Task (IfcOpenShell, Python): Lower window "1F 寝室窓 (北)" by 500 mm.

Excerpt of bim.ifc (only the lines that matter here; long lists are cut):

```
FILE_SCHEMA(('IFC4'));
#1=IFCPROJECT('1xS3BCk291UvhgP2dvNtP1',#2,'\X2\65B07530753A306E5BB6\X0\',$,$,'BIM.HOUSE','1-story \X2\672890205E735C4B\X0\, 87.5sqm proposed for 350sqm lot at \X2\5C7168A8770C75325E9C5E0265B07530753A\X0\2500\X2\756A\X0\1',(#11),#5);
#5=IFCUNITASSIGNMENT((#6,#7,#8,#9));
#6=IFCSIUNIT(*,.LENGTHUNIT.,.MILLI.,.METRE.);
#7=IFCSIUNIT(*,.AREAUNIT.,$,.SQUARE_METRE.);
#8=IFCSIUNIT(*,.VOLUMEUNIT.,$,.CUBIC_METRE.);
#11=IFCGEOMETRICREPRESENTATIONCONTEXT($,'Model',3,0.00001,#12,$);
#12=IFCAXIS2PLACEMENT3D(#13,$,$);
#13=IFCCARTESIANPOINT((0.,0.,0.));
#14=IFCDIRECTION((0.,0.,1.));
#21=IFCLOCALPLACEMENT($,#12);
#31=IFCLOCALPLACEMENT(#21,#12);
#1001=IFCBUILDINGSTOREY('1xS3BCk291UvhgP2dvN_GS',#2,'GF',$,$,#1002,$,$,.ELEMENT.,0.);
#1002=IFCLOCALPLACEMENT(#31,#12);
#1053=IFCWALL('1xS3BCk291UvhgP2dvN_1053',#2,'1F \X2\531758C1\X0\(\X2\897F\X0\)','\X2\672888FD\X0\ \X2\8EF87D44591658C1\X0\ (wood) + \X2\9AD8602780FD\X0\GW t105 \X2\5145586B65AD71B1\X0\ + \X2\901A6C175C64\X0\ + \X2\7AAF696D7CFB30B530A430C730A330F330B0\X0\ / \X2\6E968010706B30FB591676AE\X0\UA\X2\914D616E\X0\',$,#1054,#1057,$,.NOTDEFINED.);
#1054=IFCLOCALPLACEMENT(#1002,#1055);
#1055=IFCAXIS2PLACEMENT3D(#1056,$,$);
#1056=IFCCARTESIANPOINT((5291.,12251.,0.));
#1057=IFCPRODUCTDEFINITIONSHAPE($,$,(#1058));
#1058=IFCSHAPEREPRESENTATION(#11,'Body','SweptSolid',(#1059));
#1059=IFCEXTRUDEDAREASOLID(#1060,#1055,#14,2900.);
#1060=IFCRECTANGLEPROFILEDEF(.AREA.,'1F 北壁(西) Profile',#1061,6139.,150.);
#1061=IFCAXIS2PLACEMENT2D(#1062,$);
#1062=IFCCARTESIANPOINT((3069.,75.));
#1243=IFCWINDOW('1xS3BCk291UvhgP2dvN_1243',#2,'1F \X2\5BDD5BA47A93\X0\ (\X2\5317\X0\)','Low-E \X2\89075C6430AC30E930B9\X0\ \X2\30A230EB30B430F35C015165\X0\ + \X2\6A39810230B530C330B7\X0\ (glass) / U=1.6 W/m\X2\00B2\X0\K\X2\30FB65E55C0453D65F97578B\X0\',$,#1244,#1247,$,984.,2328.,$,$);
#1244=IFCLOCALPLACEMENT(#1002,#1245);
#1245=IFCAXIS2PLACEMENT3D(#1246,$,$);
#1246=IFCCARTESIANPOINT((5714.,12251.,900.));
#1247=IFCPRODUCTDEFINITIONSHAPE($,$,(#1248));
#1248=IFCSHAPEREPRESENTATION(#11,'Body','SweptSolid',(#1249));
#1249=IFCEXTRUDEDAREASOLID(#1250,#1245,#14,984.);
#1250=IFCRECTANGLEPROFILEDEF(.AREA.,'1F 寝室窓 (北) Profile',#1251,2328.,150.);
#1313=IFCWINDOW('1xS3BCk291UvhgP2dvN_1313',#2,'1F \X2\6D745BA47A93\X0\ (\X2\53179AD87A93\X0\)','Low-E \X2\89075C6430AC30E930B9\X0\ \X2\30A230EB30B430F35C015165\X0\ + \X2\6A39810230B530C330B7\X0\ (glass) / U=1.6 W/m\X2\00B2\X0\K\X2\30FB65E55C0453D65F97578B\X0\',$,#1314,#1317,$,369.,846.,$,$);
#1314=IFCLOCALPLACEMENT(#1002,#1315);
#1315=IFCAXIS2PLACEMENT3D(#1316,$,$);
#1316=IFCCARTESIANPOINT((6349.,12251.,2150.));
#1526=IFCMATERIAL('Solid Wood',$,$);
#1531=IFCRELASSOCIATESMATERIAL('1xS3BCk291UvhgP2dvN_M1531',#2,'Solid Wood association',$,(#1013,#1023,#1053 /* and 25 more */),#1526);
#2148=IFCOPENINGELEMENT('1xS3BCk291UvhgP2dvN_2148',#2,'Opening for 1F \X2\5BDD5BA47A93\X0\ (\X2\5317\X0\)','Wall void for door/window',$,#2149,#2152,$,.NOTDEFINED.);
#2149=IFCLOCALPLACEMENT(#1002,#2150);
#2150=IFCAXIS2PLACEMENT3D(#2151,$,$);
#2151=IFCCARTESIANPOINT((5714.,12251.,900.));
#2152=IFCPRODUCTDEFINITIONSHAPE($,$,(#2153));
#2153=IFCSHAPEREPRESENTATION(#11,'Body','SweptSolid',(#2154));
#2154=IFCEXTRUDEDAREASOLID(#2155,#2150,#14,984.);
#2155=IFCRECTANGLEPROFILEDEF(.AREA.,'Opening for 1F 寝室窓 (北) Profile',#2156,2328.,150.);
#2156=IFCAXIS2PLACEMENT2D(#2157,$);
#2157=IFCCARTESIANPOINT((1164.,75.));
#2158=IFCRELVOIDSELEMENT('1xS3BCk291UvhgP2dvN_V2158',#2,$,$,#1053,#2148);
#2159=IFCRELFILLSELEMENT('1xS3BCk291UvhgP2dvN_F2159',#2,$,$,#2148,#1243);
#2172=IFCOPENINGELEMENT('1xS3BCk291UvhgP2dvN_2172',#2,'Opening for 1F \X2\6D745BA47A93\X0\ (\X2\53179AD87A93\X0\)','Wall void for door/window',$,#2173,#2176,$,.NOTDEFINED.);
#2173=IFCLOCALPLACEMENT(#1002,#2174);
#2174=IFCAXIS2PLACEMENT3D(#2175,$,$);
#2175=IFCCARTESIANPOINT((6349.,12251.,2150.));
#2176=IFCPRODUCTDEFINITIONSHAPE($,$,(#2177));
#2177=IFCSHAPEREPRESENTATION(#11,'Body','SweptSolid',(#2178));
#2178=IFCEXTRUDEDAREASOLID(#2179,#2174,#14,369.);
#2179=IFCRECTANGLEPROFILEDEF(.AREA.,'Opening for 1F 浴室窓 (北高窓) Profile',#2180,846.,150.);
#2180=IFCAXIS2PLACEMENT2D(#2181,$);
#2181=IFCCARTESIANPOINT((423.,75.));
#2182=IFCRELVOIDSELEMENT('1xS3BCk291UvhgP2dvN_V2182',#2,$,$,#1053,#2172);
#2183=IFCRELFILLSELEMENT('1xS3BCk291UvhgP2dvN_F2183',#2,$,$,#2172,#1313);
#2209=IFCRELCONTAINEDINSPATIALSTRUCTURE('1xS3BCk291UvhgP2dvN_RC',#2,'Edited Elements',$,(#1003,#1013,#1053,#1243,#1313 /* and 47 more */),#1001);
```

```python
import numpy as np
import ifcopenshell
import ifcopenshell.api.geometry
import ifcopenshell.util.placement
import ifcopenshell.util.unit

model = ifcopenshell.open("bim.ifc")
unit_scale = ifcopenshell.util.unit.calculate_unit_scale(model)

window = model.by_id(1243)
opening = window.FillsVoids[0].RelatingOpeningElement
dz = -0.5 / unit_scale

shift = np.array([0.0, 0.0, dz])
# The window is not placed relative to its opening, so move both.
for product in (opening, window):
    matrix = ifcopenshell.util.placement.get_local_placement(product.ObjectPlacement)
    matrix[:3, 3] += shift
    ifcopenshell.api.geometry.edit_object_placement(model, product=product, matrix=matrix, is_si=False)

print(f"moved by {dz * unit_scale:+.3f} m")

model.write("bim_rev.ifc")
```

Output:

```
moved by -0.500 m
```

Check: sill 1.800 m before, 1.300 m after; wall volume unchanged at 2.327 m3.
